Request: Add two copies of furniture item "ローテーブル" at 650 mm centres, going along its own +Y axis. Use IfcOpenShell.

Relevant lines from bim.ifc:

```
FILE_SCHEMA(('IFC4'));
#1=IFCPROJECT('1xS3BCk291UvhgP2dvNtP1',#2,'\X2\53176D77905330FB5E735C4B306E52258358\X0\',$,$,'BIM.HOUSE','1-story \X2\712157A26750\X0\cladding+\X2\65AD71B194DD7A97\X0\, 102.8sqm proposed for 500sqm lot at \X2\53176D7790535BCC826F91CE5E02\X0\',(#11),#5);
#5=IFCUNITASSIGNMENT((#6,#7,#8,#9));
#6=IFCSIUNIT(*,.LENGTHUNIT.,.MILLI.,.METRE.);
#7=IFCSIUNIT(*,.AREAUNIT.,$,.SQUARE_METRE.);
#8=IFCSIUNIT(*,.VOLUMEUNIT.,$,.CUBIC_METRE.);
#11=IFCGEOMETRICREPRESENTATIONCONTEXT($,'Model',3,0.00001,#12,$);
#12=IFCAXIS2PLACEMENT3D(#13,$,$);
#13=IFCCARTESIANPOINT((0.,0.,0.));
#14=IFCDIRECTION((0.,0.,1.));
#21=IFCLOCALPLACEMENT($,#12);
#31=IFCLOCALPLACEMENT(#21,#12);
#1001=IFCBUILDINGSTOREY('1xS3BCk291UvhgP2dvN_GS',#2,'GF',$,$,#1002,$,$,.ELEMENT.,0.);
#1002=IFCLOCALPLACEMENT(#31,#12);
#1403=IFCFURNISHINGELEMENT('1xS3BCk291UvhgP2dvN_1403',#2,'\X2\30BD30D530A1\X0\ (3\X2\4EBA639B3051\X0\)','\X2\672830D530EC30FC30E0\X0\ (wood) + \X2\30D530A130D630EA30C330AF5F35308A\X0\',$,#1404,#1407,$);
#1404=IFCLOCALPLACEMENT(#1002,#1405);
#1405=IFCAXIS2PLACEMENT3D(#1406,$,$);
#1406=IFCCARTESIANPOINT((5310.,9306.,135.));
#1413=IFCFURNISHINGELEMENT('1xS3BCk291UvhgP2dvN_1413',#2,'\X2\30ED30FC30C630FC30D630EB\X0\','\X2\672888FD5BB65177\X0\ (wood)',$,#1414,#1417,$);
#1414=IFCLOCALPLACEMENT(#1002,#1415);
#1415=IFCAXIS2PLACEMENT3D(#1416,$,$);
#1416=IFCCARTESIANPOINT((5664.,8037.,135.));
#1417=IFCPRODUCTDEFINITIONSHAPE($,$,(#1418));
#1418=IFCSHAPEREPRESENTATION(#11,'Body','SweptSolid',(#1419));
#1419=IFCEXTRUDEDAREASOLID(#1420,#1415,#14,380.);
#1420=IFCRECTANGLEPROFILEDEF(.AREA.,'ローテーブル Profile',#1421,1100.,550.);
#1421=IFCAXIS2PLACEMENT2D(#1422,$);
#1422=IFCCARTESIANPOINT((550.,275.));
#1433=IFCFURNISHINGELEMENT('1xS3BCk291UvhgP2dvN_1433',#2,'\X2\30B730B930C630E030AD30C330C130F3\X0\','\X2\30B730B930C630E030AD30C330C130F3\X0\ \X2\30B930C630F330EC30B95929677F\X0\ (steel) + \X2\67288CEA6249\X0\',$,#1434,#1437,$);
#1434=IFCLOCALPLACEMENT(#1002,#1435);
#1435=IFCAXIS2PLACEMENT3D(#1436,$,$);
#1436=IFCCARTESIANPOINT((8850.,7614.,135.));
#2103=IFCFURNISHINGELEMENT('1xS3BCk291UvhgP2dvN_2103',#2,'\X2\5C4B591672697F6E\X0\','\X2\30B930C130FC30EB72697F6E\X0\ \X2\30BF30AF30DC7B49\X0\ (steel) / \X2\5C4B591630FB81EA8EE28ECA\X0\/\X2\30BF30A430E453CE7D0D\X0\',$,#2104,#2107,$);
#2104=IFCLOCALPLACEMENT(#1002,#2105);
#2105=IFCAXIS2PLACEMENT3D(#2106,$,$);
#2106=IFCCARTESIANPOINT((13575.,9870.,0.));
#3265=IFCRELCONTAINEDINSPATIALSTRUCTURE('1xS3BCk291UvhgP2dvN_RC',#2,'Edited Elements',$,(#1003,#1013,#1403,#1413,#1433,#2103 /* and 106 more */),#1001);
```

```python
import ifcopenshell
import ifcopenshell.api.geometry
import ifcopenshell.api.root
import ifcopenshell.util.element
import ifcopenshell.util.placement

model = ifcopenshell.open("bim.ifc")


def reuse_history(source, copy):
    """copy_class also copies each property set's owner history, people and application; keep the originals."""
    for rel in copy.IsDefinedBy:
        if rel.is_a("IfcRelDefinesByProperties") and (history := rel.RelatingPropertyDefinition.OwnerHistory):
            rel.RelatingPropertyDefinition.OwnerHistory = source.OwnerHistory
            ifcopenshell.util.element.remove_deep2(model, history)


source = model.by_guid("1xS3BCk291UvhgP2dvN_1413")
base = ifcopenshell.util.placement.get_local_placement(source.ObjectPlacement)
step = base[:3, 1] * 650.0

for i in range(1, 3):
    copy = ifcopenshell.api.root.copy_class(model, product=source)
    copy.Representation = ifcopenshell.util.element.copy_deep(
        model, source.Representation, exclude=["IfcGeometricRepresentationContext", "IfcRepresentationMap"]
    )
    reuse_history(source, copy)
    matrix = base.copy()
    matrix[:3, 3] += i * step
    print("added at", matrix[:3, 3].round(3) + 0.0)
    ifcopenshell.api.geometry.edit_object_placement(model, product=copy, matrix=matrix, is_si=False)

model.write("bim_edited.ifc")
```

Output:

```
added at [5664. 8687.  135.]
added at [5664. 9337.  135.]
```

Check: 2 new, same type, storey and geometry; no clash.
